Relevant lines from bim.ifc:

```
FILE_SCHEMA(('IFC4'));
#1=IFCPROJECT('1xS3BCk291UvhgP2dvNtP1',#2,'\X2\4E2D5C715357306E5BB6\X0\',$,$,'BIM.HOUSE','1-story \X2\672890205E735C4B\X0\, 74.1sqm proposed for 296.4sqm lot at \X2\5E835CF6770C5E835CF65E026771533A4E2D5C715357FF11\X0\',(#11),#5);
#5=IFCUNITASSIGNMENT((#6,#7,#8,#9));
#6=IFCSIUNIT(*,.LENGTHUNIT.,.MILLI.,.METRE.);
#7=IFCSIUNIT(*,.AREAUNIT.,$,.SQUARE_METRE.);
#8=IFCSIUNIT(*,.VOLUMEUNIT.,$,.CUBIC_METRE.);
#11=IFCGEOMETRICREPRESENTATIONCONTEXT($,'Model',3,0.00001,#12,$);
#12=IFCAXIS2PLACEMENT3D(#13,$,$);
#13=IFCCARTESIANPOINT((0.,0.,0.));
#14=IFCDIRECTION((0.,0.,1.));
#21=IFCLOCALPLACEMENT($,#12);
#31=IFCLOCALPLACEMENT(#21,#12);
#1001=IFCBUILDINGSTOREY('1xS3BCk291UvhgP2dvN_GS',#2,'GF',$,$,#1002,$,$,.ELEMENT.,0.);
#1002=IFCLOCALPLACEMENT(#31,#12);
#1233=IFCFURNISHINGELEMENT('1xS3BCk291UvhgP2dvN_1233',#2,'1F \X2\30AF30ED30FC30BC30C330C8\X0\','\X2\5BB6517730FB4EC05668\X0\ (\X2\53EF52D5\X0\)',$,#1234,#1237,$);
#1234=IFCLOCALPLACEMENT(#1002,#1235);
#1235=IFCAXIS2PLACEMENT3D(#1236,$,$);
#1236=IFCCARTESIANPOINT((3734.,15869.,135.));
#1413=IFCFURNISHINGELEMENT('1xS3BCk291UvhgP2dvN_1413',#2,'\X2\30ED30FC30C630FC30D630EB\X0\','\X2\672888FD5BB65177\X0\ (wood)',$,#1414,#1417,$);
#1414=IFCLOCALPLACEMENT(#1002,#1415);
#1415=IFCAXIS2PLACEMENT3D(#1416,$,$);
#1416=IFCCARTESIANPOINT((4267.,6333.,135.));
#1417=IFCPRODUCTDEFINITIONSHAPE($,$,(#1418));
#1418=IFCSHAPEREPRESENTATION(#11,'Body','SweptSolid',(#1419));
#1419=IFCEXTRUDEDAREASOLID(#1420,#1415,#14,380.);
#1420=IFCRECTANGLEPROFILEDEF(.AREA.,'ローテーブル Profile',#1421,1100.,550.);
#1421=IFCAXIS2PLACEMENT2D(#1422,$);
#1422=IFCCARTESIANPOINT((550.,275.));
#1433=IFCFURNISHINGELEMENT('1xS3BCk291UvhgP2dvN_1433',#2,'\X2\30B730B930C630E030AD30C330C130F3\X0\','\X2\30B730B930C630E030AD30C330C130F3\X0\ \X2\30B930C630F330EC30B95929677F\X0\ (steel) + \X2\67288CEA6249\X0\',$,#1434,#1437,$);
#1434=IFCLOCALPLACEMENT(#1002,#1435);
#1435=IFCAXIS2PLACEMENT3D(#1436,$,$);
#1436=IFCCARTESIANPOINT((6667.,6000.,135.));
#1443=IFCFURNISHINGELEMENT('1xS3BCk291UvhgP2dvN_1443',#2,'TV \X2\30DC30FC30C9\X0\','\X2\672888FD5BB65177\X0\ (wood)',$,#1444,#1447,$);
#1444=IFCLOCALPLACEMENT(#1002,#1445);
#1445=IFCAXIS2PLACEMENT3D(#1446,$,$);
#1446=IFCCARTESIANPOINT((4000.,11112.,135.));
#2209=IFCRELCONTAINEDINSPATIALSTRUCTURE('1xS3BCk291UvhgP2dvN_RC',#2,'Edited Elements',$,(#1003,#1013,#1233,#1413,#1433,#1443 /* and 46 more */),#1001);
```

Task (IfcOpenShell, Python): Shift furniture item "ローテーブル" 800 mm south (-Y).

```python
import ifcopenshell
import ifcopenshell.api.geometry
import ifcopenshell.util.placement
import ifcopenshell.util.unit

model = ifcopenshell.open("bim.ifc")
unit_scale = ifcopenshell.util.unit.calculate_unit_scale(model)

item = model.by_guid("1xS3BCk291UvhgP2dvN_1413")
matrix = ifcopenshell.util.placement.get_local_placement(item.ObjectPlacement)
matrix[1, 3] -= 0.8 / unit_scale
ifcopenshell.api.geometry.edit_object_placement(model, product=item, matrix=matrix, is_si=False)

print(ifcopenshell.util.placement.get_local_placement(item.ObjectPlacement).round(3) + 0.0)

model.write("bim_v2.ifc")
```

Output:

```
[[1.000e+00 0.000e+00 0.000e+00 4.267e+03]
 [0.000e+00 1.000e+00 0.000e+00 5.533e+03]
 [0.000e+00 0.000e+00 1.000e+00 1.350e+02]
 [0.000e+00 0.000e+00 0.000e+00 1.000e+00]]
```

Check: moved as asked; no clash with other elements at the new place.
